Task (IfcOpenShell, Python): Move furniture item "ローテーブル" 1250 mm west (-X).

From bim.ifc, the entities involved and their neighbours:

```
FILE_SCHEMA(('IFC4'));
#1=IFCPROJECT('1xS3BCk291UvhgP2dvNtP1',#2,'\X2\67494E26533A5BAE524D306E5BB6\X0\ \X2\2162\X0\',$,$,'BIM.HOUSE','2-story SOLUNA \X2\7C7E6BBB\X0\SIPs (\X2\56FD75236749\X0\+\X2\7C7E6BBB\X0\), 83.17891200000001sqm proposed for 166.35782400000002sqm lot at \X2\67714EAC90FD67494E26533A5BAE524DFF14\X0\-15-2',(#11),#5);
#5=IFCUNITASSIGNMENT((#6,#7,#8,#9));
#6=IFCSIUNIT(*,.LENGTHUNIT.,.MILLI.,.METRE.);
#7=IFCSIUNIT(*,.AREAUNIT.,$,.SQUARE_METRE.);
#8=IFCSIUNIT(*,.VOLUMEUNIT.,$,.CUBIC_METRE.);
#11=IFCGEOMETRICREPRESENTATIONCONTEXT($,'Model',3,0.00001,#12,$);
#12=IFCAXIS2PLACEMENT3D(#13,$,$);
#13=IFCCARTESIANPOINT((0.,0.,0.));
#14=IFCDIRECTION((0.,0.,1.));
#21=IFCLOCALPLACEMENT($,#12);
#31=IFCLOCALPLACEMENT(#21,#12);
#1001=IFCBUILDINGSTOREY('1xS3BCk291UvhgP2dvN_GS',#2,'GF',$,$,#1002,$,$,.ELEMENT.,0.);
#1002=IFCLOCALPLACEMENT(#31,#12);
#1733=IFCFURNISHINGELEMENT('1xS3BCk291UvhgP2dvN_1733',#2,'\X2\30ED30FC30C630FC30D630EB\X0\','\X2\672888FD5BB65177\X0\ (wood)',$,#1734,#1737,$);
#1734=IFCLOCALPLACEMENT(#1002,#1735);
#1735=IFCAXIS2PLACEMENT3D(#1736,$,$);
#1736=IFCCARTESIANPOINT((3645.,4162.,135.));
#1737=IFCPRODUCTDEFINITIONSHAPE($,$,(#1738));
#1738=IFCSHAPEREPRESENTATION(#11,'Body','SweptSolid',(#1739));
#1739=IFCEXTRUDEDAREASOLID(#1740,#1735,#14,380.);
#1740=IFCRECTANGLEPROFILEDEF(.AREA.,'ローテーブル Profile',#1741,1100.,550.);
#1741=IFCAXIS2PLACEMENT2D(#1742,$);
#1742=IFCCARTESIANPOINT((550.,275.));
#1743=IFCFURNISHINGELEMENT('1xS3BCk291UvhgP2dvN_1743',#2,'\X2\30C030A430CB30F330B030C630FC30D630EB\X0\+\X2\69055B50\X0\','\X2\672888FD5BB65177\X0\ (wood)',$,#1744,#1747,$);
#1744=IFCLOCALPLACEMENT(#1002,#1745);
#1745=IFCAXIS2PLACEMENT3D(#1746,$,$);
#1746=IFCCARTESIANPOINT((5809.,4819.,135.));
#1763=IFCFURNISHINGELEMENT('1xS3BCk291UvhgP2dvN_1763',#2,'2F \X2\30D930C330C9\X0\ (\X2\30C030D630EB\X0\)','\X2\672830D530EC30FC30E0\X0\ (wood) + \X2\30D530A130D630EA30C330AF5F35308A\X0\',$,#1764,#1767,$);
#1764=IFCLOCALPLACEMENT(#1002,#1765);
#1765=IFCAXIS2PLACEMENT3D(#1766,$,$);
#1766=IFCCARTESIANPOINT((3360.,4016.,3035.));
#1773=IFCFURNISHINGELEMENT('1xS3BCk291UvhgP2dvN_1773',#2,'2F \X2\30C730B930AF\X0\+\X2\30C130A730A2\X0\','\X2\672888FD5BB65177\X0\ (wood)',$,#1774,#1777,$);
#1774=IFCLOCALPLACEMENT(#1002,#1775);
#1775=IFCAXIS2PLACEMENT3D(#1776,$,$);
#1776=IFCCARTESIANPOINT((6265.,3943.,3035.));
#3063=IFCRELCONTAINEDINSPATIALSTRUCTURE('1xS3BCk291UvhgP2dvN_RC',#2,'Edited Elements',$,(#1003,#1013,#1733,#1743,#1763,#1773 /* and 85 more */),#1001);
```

```python
import ifcopenshell
import ifcopenshell.api.geometry
import ifcopenshell.util.placement
import ifcopenshell.util.unit

model = ifcopenshell.open("bim.ifc")
unit_scale = ifcopenshell.util.unit.calculate_unit_scale(model)

item = model.by_guid("1xS3BCk291UvhgP2dvN_1733")
matrix = ifcopenshell.util.placement.get_local_placement(item.ObjectPlacement)
matrix[0, 3] -= 1.25 / unit_scale
ifcopenshell.api.geometry.edit_object_placement(model, product=item, matrix=matrix, is_si=False)

print(ifcopenshell.util.placement.get_local_placement(item.ObjectPlacement).round(3) + 0.0)

model.write("bim_v2.ifc")
```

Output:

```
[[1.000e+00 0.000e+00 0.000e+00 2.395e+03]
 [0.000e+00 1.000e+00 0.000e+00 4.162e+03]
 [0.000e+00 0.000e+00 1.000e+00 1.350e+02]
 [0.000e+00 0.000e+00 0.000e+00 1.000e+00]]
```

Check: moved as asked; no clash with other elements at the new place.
